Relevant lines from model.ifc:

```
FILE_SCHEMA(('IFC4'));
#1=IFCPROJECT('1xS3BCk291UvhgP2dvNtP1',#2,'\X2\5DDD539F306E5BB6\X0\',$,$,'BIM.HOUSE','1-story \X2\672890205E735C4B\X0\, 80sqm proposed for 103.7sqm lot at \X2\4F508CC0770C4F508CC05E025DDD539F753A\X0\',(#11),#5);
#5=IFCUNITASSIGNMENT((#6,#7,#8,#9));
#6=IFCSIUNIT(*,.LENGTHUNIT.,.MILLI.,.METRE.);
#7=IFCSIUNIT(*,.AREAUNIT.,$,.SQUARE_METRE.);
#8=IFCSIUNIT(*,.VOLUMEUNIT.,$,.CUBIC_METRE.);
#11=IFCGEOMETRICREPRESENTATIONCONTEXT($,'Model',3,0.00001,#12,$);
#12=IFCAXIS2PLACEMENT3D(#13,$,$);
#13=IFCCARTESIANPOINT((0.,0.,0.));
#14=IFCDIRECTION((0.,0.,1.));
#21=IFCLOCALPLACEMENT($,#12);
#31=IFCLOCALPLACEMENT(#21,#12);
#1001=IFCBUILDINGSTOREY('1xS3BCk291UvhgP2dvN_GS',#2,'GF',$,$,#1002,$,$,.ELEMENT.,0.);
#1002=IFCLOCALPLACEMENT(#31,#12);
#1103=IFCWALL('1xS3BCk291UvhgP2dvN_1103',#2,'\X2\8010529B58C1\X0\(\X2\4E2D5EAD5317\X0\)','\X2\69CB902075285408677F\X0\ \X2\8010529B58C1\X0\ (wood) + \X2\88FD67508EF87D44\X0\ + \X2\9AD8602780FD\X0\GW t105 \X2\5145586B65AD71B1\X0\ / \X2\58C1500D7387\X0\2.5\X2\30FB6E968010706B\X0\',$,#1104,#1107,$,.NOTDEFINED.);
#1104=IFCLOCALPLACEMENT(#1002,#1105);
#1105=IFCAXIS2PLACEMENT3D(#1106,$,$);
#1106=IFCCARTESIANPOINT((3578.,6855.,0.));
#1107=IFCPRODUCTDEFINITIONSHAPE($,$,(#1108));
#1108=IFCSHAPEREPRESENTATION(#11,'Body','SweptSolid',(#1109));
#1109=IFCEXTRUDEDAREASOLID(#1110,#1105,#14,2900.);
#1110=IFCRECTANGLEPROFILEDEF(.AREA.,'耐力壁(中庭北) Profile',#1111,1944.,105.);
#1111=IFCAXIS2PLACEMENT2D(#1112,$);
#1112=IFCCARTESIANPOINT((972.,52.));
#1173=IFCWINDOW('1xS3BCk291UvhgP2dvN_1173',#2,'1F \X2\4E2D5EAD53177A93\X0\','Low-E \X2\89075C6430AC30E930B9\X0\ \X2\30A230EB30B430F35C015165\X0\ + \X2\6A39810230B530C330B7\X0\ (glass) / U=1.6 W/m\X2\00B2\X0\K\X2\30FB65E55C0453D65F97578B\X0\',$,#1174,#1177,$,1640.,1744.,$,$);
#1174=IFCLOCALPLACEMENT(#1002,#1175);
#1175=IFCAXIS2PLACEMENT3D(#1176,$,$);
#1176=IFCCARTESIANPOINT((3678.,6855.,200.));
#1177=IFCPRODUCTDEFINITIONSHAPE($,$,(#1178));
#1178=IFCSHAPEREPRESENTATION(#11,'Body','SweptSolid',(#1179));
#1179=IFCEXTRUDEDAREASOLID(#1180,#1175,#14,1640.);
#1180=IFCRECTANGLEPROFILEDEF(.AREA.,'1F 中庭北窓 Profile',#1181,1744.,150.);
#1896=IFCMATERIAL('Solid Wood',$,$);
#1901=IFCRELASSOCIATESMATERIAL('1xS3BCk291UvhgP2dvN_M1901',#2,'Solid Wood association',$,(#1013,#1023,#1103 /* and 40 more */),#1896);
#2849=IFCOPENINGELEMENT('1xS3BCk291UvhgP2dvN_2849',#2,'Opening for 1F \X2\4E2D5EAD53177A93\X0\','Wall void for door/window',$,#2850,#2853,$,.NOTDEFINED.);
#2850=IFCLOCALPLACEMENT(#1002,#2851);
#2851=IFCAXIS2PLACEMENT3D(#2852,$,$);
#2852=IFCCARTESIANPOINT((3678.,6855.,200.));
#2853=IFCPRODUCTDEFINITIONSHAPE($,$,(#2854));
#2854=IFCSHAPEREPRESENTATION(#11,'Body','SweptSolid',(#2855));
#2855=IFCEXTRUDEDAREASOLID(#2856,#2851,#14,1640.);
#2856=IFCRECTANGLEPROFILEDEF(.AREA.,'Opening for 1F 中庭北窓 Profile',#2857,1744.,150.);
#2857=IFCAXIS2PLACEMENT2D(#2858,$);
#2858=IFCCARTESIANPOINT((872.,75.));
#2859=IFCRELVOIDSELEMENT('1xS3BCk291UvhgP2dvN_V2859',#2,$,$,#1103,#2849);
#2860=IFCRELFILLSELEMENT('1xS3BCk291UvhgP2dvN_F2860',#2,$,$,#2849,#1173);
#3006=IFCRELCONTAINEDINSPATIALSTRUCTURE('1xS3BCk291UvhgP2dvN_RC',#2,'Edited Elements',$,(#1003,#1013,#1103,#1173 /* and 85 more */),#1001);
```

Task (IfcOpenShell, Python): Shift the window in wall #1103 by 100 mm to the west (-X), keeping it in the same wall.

```python
import ifcopenshell
import ifcopenshell.api.geometry
import ifcopenshell.util.placement
import ifcopenshell.util.unit

model = ifcopenshell.open("model.ifc")
unit_scale = ifcopenshell.util.unit.calculate_unit_scale(model)

window = model.by_id(1173)
opening = window.FillsVoids[0].RelatingOpeningElement
wall = opening.VoidsElements[0].RelatingBuildingElement

wall_matrix = ifcopenshell.util.placement.get_local_placement(wall.ObjectPlacement)
shift = wall_matrix[:3, 0] * -0.1 / unit_scale
before = ifcopenshell.util.placement.get_local_placement(window.ObjectPlacement)[:3, 3].copy()

# The window is not placed relative to its opening, so move both.
for product in (opening, window):
    matrix = ifcopenshell.util.placement.get_local_placement(product.ObjectPlacement)
    matrix[:3, 3] += shift
    ifcopenshell.api.geometry.edit_object_placement(model, product=product, matrix=matrix, is_si=False)

after = ifcopenshell.util.placement.get_local_placement(window.ObjectPlacement)[:3, 3]
print("window moved by", (after - before).round(3) + 0.0)

model.write("model_v2.ifc")
```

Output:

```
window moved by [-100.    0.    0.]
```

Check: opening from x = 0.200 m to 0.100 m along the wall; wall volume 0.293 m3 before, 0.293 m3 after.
